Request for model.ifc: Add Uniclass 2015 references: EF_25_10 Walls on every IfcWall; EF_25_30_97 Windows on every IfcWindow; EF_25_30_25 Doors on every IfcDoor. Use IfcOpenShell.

First a look at what the model holds.

```python
import ifcopenshell

model = ifcopenshell.open("model.ifc")
print(model.schema)
print("classifications:", [c.Name for c in model.by_type("IfcClassification")])
for ifc_class in ("IfcDoor", "IfcRoof", "IfcStair", "IfcWall", "IfcWindow"):
    print(ifc_class, len(model.by_type(ifc_class)))
```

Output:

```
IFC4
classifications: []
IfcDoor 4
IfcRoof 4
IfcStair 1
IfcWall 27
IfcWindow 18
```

```python
import ifcopenshell
import ifcopenshell.api.classification

model = ifcopenshell.open("model.ifc")

system = ifcopenshell.api.classification.add_classification(model, classification="Uniclass 2015")

codes = {
    "IfcWall": ("EF_25_10", "Walls"),
    "IfcWindow": ("EF_25_30_97", "Windows"),
    "IfcDoor": ("EF_25_30_25", "Doors"),
}
for ifc_class, (code, name) in codes.items():
    products = model.by_type(ifc_class)
    ifcopenshell.api.classification.add_reference(
        model, products=products, classification=system, identification=code, name=name
    )
    print(code, len(products))

model.write("model-out.ifc")
```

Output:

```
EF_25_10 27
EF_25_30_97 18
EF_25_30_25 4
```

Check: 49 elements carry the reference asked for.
